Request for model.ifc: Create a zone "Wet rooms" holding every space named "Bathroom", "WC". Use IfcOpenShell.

First a look at what the model holds.

```python
import ifcopenshell

model = ifcopenshell.open("model.ifc")
print(model.schema)
seen = {}
for space in model.by_type("IfcSpace"):
    seen[space.LongName] = seen.get(space.LongName, 0) + 1
for name, count in sorted(seen.items(), key=str):
    print(count, "x", name)
print("zones:", [z.Name for z in model.by_type("IfcZone")][:20])
```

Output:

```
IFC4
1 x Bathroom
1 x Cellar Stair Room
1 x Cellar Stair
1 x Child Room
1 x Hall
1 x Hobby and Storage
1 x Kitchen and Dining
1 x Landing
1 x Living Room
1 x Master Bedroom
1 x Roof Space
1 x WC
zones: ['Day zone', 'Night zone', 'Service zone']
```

```python
import ifcopenshell
import ifcopenshell.api.group
import ifcopenshell.api.root

model = ifcopenshell.open("model.ifc")

names = {"Bathroom", "WC"}
spaces = [s for s in model.by_type("IfcSpace") if s.LongName in names]

zone = ifcopenshell.api.root.create_entity(model, ifc_class="IfcZone", name="Wet rooms")
ifcopenshell.api.group.assign_group(model, products=spaces, group=zone)
print(len(spaces), "spaces in", zone.Name)

model.write("model_rev.ifc")
```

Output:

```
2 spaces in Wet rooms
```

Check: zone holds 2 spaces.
